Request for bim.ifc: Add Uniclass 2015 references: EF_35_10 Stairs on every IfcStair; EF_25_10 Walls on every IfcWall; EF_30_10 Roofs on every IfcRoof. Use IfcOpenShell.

First a look at what the model holds.

```python
import ifcopenshell

model = ifcopenshell.open("bim.ifc")
print(model.schema)
print("classifications:", [c.Name for c in model.by_type("IfcClassification")])
for ifc_class in ("IfcDoor", "IfcRoof", "IfcStair", "IfcWall", "IfcWindow"):
    print(ifc_class, len(model.by_type(ifc_class)))
```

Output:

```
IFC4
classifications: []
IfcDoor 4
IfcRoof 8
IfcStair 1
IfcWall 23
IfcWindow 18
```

```python
import ifcopenshell
import ifcopenshell.api.classification

model = ifcopenshell.open("bim.ifc")

system = ifcopenshell.api.classification.add_classification(model, classification="Uniclass 2015")

codes = {
    "IfcStair": ("EF_35_10", "Stairs"),
    "IfcWall": ("EF_25_10", "Walls"),
    "IfcRoof": ("EF_30_10", "Roofs"),
}
for ifc_class, (code, name) in codes.items():
    products = model.by_type(ifc_class)
    ifcopenshell.api.classification.add_reference(
        model, products=products, classification=system, identification=code, name=name
    )
    print(code, len(products))

model.write("bim-out.ifc")
```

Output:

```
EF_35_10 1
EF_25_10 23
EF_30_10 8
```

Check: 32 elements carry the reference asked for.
